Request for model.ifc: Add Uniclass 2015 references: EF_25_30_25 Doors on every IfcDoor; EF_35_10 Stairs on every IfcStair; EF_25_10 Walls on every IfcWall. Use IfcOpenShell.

First a look at what the model holds.

```python
import ifcopenshell

model = ifcopenshell.open("model.ifc")
print(model.schema)
print("classifications:", [c.Name for c in model.by_type("IfcClassification")])
for ifc_class in ("IfcDoor", "IfcRoof", "IfcStair", "IfcWall", "IfcWindow"):
    print(ifc_class, len(model.by_type(ifc_class)))
```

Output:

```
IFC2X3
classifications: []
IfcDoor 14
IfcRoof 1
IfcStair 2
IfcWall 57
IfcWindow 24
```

```python
import ifcopenshell
import ifcopenshell.api.classification

model = ifcopenshell.open("model.ifc")

# IFC2X3 requires Source and Edition and has no link from the project to the system.
system = model.create_entity("IfcClassification", Source="NBS", Edition="2015", Name="Uniclass 2015")

codes = {
    "IfcDoor": ("EF_25_30_25", "Doors"),
    "IfcStair": ("EF_35_10", "Stairs"),
    "IfcWall": ("EF_25_10", "Walls"),
}
for ifc_class, (code, name) in codes.items():
    products = model.by_type(ifc_class)
    ifcopenshell.api.classification.add_reference(
        model, products=products, classification=system, identification=code, name=name
    )
    print(code, len(products))

model.write("model_v2.ifc")
```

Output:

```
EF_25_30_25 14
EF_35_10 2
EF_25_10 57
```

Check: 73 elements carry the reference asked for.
